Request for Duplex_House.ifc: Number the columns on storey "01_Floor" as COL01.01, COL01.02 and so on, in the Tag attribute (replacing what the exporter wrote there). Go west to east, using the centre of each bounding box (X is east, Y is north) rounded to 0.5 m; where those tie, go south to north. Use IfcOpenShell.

First a look at what the model holds.

```python
import ifcopenshell
import ifcopenshell.util.element
import ifcopenshell.util.placement

model = ifcopenshell.open("Duplex_House.ifc")
print(model.schema)
storey = next(s for s in model.by_type("IfcBuildingStorey") if s.Name == "01_Floor")
columns = [e for e in ifcopenshell.util.element.get_decomposition(storey) if e.is_a("IfcColumn")]
for e in sorted(columns, key=lambda e: e.id()):
    origin = ifcopenshell.util.placement.get_local_placement(e.ObjectPlacement)[:3, 3]
    print(e.id(), e.Tag, e.Name, origin.round(2) + 0.0, sep=" | ")
```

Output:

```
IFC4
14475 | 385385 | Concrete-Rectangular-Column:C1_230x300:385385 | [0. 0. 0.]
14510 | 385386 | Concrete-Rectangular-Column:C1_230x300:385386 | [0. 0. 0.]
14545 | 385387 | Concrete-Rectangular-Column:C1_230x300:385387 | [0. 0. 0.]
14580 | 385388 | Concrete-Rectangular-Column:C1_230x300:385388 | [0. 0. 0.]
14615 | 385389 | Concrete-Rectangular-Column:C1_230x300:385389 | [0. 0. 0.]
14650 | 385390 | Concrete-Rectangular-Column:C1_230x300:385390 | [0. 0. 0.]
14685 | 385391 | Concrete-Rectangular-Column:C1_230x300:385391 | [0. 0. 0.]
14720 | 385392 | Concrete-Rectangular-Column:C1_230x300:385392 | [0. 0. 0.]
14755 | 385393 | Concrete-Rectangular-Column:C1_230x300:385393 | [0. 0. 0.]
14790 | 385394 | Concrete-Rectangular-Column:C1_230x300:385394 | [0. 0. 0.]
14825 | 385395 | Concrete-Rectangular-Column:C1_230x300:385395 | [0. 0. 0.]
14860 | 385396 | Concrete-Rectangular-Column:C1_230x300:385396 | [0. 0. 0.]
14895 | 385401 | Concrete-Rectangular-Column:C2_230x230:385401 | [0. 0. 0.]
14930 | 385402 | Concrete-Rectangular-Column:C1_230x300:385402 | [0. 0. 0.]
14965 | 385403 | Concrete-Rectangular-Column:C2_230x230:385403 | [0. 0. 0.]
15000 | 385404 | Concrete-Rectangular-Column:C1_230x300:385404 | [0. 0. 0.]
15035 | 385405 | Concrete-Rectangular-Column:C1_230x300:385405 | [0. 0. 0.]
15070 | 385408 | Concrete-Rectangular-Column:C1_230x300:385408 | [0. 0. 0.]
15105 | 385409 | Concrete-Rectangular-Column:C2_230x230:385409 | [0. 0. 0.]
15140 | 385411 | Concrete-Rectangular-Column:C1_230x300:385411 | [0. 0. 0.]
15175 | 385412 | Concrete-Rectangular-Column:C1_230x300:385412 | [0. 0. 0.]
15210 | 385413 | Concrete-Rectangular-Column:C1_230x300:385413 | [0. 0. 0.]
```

```python
import ifcopenshell
import ifcopenshell.geom
import ifcopenshell.util.element
import ifcopenshell.util.shape

model = ifcopenshell.open("Duplex_House.ifc")
settings = ifcopenshell.geom.settings()
settings.set("use-world-coords", True)


def centre(element):
    shape = ifcopenshell.geom.create_shape(settings, element)
    return ifcopenshell.util.shape.get_bbox_centroid(shape.geometry)


storey = next(s for s in model.by_type("IfcBuildingStorey") if s.Name == "01_Floor")
columns = [e for e in ifcopenshell.util.element.get_decomposition(storey) if e.is_a("IfcColumn")]

# Insertion points can sit at a corner or the storey origin, so sort by the geometry (in metres).
centres = {e: centre(e) for e in columns}
columns.sort(key=lambda e: (round(centres[e][0] / 0.5), centres[e][1]))

for i, e in enumerate(columns, start=1):
    number = f"COL01.{i:02d}"
    e.Tag = number
    print(e.id(), number)

model.write("Duplex_House-out.ifc")
```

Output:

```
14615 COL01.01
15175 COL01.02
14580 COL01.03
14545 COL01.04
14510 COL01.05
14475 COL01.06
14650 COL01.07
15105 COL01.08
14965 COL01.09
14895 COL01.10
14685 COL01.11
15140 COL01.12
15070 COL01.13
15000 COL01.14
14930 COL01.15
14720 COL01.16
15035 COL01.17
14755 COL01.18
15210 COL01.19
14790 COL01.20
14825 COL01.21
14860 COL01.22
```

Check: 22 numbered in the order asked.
